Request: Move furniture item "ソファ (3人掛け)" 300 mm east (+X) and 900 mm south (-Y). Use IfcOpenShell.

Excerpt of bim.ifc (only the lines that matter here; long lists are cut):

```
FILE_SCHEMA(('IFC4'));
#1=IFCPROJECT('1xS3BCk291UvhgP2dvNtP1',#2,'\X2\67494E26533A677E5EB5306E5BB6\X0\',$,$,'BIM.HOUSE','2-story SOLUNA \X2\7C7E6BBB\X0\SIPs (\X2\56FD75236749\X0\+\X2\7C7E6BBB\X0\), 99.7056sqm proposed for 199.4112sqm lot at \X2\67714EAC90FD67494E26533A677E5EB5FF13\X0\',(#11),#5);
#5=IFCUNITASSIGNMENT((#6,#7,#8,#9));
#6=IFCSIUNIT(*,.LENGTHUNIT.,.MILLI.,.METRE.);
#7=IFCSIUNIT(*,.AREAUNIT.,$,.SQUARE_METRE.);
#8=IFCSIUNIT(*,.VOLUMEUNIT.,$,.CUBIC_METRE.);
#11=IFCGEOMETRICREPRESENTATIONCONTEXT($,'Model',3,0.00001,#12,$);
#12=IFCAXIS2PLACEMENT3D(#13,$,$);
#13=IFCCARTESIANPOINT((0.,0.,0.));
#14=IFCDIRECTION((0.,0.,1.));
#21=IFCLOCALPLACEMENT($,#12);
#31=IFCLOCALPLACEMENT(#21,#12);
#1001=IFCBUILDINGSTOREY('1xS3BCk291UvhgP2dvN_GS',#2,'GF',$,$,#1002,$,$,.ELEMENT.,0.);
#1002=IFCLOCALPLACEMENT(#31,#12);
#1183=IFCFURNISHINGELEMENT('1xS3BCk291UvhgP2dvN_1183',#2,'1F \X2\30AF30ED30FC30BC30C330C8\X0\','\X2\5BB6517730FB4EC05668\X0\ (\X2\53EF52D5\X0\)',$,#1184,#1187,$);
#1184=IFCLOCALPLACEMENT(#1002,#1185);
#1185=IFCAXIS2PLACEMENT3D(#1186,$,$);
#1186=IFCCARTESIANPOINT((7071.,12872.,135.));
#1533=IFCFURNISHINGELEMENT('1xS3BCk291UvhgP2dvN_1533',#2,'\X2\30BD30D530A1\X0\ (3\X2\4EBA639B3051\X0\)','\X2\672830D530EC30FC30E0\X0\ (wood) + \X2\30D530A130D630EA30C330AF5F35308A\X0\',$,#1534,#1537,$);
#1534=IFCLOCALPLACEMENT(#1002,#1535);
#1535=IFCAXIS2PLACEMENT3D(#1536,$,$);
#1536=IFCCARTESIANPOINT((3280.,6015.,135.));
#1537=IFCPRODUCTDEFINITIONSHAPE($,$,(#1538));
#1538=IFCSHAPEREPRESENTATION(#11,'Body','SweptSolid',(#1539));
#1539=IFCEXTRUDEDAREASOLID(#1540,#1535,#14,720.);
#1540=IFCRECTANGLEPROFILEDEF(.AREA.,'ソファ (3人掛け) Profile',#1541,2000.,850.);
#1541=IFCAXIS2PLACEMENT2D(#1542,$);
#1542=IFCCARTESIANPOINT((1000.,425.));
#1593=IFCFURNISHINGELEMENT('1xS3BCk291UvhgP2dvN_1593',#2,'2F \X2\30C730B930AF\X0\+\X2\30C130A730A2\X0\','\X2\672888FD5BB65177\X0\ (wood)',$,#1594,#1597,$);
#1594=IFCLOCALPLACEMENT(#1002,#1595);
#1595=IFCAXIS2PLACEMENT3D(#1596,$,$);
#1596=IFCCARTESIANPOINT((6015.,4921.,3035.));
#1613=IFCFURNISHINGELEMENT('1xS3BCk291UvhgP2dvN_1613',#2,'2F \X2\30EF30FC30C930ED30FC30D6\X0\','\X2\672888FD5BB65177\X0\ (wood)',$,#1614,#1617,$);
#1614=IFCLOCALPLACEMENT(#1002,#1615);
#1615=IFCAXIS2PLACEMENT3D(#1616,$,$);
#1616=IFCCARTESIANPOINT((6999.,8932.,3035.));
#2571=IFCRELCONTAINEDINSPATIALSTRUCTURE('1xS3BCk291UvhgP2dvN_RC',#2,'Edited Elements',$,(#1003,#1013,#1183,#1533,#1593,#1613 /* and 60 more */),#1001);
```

```python
import ifcopenshell
import ifcopenshell.api.geometry
import ifcopenshell.util.placement
import ifcopenshell.util.unit

model = ifcopenshell.open("bim.ifc")
unit_scale = ifcopenshell.util.unit.calculate_unit_scale(model)

item = model.by_guid("1xS3BCk291UvhgP2dvN_1533")
matrix = ifcopenshell.util.placement.get_local_placement(item.ObjectPlacement)
matrix[0, 3] += 0.3 / unit_scale
matrix[1, 3] -= 0.9 / unit_scale
ifcopenshell.api.geometry.edit_object_placement(model, product=item, matrix=matrix, is_si=False)

print(ifcopenshell.util.placement.get_local_placement(item.ObjectPlacement).round(3) + 0.0)

model.write("bim-out.ifc")
```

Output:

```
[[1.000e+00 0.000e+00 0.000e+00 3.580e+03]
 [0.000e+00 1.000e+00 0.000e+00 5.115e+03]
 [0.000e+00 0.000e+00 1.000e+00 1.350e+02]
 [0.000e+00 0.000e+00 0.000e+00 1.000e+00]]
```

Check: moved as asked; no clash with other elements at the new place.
